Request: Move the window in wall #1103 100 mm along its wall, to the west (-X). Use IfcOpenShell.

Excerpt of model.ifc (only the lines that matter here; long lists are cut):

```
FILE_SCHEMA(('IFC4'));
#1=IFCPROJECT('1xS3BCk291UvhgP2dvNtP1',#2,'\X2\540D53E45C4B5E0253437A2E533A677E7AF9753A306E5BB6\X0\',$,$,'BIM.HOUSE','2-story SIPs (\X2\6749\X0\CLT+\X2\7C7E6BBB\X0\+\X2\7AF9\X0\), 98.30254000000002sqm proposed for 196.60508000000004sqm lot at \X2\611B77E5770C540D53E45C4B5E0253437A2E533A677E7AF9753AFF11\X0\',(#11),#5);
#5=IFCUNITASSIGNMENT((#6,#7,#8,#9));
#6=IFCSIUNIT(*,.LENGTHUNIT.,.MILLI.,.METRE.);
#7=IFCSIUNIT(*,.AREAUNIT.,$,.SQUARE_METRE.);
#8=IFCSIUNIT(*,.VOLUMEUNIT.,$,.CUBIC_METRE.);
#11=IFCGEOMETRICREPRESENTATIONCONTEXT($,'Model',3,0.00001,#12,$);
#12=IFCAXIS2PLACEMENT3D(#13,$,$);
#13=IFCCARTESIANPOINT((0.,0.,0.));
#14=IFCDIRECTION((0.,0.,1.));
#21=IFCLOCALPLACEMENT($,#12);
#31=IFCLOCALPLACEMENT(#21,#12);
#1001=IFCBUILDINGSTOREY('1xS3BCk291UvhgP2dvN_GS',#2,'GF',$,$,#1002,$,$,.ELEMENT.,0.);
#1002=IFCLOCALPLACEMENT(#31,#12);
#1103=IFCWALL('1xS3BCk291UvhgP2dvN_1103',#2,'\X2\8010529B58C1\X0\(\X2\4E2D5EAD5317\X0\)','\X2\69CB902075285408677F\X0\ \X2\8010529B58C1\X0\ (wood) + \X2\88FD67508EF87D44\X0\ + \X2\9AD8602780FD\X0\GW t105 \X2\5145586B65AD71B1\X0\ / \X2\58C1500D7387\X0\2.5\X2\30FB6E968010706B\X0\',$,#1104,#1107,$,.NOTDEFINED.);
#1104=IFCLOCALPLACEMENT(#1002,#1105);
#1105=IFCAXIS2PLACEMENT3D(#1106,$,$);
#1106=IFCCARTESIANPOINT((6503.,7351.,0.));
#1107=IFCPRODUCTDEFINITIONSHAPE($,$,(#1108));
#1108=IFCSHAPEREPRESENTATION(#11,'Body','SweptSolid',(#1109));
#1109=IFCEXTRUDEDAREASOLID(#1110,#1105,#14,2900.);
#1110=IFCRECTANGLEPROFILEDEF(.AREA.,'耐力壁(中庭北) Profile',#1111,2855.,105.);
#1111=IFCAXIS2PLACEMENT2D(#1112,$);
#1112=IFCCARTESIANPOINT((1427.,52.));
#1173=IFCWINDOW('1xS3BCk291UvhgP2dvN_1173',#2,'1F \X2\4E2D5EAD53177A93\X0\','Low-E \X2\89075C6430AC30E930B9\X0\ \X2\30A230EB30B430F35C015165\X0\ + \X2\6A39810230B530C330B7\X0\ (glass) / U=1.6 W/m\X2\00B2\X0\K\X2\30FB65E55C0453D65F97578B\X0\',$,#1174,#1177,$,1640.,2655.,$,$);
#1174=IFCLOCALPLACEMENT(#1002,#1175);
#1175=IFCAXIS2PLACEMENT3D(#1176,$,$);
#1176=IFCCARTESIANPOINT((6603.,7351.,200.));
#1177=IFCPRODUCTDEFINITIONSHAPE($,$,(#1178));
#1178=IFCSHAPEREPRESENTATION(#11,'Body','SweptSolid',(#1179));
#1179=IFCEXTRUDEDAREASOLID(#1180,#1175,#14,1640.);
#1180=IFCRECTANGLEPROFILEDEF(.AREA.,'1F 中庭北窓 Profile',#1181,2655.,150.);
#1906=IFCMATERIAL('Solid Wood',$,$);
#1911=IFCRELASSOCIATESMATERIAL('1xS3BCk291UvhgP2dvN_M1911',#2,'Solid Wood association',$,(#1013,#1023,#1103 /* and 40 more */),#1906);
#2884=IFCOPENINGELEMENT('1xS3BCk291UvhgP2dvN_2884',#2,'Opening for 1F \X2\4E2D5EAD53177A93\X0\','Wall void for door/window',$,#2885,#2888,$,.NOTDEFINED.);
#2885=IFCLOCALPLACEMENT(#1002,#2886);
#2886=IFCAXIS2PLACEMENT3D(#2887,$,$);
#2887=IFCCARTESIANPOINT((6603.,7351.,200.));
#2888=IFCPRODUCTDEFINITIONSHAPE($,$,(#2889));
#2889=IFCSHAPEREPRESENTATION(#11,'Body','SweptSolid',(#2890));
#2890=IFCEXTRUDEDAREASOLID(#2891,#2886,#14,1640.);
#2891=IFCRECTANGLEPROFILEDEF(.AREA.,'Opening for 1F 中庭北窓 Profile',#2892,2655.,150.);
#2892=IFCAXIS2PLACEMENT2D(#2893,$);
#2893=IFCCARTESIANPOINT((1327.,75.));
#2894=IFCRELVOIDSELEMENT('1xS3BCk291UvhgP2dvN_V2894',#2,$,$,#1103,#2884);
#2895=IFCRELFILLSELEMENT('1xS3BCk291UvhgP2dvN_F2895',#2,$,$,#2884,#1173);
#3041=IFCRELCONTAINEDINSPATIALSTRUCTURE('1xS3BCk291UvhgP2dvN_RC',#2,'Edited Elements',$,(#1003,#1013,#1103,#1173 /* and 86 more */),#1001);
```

```python
import ifcopenshell
import ifcopenshell.api.geometry
import ifcopenshell.util.placement
import ifcopenshell.util.unit

model = ifcopenshell.open("model.ifc")
unit_scale = ifcopenshell.util.unit.calculate_unit_scale(model)

window = model.by_guid("1xS3BCk291UvhgP2dvN_1173")
opening = window.FillsVoids[0].RelatingOpeningElement
wall = opening.VoidsElements[0].RelatingBuildingElement

wall_matrix = ifcopenshell.util.placement.get_local_placement(wall.ObjectPlacement)
shift = wall_matrix[:3, 0] * -0.1 / unit_scale
before = ifcopenshell.util.placement.get_local_placement(window.ObjectPlacement)[:3, 3].copy()

# The window is not placed relative to its opening, so move both.
for product in (opening, window):
    matrix = ifcopenshell.util.placement.get_local_placement(product.ObjectPlacement)
    matrix[:3, 3] += shift
    ifcopenshell.api.geometry.edit_object_placement(model, product=product, matrix=matrix, is_si=False)

after = ifcopenshell.util.placement.get_local_placement(window.ObjectPlacement)[:3, 3]
print("window moved by", (after - before).round(3) + 0.0)

model.write("model_edited.ifc")
```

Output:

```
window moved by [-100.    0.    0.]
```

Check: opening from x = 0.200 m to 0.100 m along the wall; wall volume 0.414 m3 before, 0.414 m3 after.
